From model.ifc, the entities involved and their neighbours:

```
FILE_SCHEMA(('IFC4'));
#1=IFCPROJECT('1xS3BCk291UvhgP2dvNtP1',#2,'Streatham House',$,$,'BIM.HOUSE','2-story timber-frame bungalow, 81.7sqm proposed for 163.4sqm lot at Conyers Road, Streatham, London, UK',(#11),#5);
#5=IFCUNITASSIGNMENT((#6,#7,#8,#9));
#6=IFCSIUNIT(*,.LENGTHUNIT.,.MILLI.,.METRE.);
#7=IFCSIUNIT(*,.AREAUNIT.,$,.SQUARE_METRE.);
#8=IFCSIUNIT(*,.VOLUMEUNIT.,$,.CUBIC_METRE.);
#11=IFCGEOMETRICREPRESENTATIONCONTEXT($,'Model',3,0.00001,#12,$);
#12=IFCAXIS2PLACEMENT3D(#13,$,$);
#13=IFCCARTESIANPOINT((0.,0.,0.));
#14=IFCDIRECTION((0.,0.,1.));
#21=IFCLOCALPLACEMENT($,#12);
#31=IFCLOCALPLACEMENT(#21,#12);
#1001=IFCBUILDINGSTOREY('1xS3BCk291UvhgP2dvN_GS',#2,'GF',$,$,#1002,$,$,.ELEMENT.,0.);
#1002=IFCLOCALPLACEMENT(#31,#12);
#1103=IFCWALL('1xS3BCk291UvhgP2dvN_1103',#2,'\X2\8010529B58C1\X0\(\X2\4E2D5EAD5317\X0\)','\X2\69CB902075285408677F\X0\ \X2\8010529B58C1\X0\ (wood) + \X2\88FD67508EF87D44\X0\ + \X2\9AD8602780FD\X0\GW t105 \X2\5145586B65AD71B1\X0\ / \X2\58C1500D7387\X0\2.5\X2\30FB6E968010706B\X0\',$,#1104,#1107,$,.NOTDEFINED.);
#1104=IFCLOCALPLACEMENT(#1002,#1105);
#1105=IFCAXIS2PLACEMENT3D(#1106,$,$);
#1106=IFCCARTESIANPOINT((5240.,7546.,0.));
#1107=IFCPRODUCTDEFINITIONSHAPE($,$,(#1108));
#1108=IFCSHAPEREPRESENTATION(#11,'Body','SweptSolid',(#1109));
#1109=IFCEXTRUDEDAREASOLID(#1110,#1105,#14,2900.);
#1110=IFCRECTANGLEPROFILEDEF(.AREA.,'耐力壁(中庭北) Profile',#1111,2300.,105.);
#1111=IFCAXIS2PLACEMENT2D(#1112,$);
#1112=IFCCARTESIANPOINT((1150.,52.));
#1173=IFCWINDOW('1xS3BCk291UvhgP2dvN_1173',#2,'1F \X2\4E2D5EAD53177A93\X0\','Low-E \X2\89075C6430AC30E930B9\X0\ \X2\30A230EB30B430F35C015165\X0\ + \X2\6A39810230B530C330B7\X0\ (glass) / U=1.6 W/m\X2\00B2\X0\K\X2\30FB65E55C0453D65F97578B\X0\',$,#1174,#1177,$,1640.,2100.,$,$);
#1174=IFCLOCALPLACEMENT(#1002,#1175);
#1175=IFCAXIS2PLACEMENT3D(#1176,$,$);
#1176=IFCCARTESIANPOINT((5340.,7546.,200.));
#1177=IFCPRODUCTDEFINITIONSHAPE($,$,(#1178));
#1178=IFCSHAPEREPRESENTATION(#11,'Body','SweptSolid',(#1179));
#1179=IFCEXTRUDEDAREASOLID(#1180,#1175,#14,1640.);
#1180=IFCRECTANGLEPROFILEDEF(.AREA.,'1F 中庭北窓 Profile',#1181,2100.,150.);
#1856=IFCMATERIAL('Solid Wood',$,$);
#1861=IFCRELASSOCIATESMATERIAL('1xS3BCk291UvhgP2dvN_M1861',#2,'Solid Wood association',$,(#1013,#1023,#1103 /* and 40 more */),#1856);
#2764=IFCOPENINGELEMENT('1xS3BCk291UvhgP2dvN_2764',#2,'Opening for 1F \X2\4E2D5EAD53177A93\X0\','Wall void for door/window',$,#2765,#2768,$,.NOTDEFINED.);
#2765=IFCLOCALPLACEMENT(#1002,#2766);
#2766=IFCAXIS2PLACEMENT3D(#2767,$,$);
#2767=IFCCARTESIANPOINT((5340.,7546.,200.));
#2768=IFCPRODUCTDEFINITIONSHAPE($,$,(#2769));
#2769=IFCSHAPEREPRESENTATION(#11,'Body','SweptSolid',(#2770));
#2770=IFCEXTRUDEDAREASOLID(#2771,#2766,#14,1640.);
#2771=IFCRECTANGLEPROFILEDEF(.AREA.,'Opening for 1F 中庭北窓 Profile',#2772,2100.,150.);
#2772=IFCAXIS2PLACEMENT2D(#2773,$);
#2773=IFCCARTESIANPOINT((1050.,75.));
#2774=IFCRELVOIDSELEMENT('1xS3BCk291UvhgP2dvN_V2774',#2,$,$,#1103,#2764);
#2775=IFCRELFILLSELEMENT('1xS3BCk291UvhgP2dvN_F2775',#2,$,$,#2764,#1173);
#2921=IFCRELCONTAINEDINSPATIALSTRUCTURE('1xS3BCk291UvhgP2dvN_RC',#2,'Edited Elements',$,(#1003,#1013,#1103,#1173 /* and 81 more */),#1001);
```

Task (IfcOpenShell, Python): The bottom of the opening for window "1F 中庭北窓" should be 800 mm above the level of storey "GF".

```python
import numpy as np
import ifcopenshell
import ifcopenshell.api.geometry
import ifcopenshell.geom
import ifcopenshell.util.element
import ifcopenshell.util.placement
import ifcopenshell.util.shape
import ifcopenshell.util.unit

model = ifcopenshell.open("model.ifc")
unit_scale = ifcopenshell.util.unit.calculate_unit_scale(model)

window = model.by_guid("1xS3BCk291UvhgP2dvN_1173")
opening = window.FillsVoids[0].RelatingOpeningElement
storey = ifcopenshell.util.element.get_container(window, ifc_class="IfcBuildingStorey")
level = ifcopenshell.util.placement.get_local_placement(storey.ObjectPlacement)[2, 3]

# The opening's origin need not be at the sill, so measure its lowest point.
shape = ifcopenshell.geom.create_shape(ifcopenshell.geom.settings(), opening)
bottom = ifcopenshell.util.shape.get_shape_bottom_elevation(shape, shape.geometry) / unit_scale
dz = level + 0.8 / unit_scale - bottom

shift = np.array([0.0, 0.0, dz])
# The window is not placed relative to its opening, so move both.
for product in (opening, window):
    matrix = ifcopenshell.util.placement.get_local_placement(product.ObjectPlacement)
    matrix[:3, 3] += shift
    ifcopenshell.api.geometry.edit_object_placement(model, product=product, matrix=matrix, is_si=False)

print(f"moved by {dz * unit_scale:+.3f} m")

model.write("model_updated.ifc")
```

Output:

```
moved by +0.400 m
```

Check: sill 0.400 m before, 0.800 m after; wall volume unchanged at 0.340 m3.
